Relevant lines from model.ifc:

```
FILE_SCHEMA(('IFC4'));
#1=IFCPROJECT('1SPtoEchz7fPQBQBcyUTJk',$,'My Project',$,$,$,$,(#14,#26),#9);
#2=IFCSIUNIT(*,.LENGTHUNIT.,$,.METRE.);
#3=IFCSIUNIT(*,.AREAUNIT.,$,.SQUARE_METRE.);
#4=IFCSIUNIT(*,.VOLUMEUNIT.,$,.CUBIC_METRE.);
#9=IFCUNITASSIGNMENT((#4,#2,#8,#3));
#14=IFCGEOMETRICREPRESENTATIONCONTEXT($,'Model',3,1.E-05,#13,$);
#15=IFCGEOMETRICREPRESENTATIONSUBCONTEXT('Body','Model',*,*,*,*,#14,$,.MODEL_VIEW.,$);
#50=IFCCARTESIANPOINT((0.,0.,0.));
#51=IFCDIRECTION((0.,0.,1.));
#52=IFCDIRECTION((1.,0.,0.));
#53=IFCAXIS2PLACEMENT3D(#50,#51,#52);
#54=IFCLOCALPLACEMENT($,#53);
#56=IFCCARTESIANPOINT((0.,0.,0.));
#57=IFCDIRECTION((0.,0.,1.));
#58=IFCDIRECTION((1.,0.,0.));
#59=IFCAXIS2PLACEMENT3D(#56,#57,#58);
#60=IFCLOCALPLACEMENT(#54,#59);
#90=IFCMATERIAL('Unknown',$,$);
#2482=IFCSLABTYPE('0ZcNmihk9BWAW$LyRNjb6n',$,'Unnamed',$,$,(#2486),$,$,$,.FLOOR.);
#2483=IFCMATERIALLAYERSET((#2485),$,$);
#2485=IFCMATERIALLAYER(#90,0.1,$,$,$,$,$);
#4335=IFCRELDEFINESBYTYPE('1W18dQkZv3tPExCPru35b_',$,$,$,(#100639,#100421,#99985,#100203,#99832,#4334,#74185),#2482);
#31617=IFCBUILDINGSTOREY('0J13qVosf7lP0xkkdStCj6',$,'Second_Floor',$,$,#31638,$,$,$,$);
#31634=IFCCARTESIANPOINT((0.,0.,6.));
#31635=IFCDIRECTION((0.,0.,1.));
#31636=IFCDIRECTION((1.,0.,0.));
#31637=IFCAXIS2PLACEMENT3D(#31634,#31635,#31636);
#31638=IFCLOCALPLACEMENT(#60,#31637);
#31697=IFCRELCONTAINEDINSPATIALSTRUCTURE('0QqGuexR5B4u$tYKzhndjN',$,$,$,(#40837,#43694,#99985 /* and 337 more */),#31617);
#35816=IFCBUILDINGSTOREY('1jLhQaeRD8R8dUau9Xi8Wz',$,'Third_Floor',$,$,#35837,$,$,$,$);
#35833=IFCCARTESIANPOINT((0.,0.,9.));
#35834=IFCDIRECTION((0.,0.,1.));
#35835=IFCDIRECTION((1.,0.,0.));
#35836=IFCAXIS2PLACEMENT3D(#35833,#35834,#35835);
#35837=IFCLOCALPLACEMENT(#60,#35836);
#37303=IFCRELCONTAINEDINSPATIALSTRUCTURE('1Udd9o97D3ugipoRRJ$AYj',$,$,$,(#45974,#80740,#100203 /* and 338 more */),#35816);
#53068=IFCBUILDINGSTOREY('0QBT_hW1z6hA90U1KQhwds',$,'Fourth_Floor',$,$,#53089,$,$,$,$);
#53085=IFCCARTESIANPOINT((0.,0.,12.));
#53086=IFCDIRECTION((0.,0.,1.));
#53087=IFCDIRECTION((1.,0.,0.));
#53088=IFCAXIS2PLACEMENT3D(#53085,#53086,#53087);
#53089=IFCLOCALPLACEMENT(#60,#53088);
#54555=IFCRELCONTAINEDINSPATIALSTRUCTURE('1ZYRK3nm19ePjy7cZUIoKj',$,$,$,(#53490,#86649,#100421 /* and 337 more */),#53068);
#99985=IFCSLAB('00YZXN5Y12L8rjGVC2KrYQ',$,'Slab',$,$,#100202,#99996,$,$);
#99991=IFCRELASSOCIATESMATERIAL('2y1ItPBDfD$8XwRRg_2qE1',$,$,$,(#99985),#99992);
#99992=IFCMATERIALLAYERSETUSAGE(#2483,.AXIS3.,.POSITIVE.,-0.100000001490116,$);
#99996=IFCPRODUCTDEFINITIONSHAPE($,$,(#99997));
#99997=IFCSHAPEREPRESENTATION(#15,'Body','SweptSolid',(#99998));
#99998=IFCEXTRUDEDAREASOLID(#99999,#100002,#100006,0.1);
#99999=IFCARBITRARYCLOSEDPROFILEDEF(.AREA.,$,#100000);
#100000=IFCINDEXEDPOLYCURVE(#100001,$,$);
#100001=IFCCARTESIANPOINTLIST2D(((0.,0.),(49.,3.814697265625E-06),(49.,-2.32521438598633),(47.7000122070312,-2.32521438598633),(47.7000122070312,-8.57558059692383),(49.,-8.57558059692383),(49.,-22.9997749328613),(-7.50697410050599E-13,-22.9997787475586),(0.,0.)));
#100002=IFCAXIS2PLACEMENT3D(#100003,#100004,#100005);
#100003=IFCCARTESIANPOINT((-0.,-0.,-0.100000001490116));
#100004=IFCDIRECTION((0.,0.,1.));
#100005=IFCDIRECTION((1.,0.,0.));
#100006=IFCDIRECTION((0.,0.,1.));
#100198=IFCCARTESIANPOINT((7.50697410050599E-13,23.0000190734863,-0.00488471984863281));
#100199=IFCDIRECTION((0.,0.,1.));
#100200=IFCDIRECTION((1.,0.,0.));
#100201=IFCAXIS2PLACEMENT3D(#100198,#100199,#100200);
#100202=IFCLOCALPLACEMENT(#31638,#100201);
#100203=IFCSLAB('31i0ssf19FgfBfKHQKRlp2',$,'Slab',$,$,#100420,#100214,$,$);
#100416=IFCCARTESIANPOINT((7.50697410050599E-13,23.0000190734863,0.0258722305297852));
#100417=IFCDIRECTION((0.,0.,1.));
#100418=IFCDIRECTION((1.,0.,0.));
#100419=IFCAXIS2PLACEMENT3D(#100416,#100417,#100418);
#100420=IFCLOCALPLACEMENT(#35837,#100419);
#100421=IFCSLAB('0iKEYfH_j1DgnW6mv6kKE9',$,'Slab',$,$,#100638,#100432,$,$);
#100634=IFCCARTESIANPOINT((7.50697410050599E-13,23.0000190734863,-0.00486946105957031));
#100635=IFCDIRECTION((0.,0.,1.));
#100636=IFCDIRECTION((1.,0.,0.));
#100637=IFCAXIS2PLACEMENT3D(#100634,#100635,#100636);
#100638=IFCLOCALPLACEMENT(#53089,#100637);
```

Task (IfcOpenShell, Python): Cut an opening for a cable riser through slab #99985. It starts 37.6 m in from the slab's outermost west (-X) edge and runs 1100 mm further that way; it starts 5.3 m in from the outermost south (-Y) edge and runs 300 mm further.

```python
import numpy as np
import ifcopenshell
import ifcopenshell.api.feature
import ifcopenshell.api.geometry
import ifcopenshell.api.root
import ifcopenshell.geom
import ifcopenshell.util.placement
import ifcopenshell.util.representation
import ifcopenshell.util.shape
import ifcopenshell.util.unit

model = ifcopenshell.open("model.ifc")
unit_scale = ifcopenshell.util.unit.calculate_unit_scale(model)
settings = ifcopenshell.geom.settings()


def volume(element):
    """Net volume in cubic metres, openings subtracted."""
    shape = ifcopenshell.geom.create_shape(settings, element)
    return ifcopenshell.util.shape.get_volume(shape.geometry)


slab = model.by_guid("00YZXN5Y12L8rjGVC2KrYQ")
before = volume(slab)

# Extent in the slab's own axes, in metres. The edges named are its -X and -Y sides.
slab_shape = ifcopenshell.geom.create_shape(settings, slab)
vertices = ifcopenshell.util.shape.get_vertices(slab_shape.geometry)
x_min, y_min, bottom = vertices.min(axis=0)
top = vertices[:, 2].max()

opening = ifcopenshell.api.root.create_entity(model, ifc_class="IfcOpeningElement", name="Cable riser opening", predefined_type="OPENING")
context = ifcopenshell.util.representation.get_context(model, "Model", "Body", "MODEL_VIEW")
width, depth = 1.1, 0.3
outline = [(0.0, 0.0), (width, 0.0), (width, depth), (0.0, depth), (0.0, 0.0)]
# Overshoot both faces by 50 mm so the cut is clean.
shape = ifcopenshell.api.geometry.add_slab_representation(
    model, context=context, depth=top - bottom + 0.1, polyline=outline
)
ifcopenshell.api.geometry.assign_representation(model, product=opening, representation=shape)

matrix = ifcopenshell.util.placement.get_local_placement(slab.ObjectPlacement)
matrix[:, 3] = matrix @ np.append(np.array([x_min + 37.6, y_min + 5.3, bottom - 0.05]) / unit_scale, 1.0)
ifcopenshell.api.geometry.edit_object_placement(model, product=opening, matrix=matrix, is_si=False)
ifcopenshell.api.feature.add_feature(model, feature=opening, element=slab)

after = volume(slab)

print(f"slab volume {before:.3f} -> {after:.3f} m3")

model.write("model_edited.ifc")
```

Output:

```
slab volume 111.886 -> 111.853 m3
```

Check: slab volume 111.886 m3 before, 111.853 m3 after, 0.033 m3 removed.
